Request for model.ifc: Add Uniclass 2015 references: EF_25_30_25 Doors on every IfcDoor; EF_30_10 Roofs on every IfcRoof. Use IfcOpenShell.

First a look at what the model holds.

```python
import ifcopenshell

model = ifcopenshell.open("model.ifc")
print(model.schema)
print("classifications:", [c.Name for c in model.by_type("IfcClassification")])
for ifc_class in ("IfcDoor", "IfcRoof", "IfcStair", "IfcWall", "IfcWindow"):
    print(ifc_class, len(model.by_type(ifc_class)))
```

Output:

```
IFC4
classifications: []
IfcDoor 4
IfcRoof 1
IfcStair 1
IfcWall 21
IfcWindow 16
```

```python
import ifcopenshell
import ifcopenshell.api.classification

model = ifcopenshell.open("model.ifc")

system = ifcopenshell.api.classification.add_classification(model, classification="Uniclass 2015")

codes = {
    "IfcDoor": ("EF_25_30_25", "Doors"),
    "IfcRoof": ("EF_30_10", "Roofs"),
}
for ifc_class, (code, name) in codes.items():
    products = model.by_type(ifc_class)
    ifcopenshell.api.classification.add_reference(
        model, products=products, classification=system, identification=code, name=name
    )
    print(code, len(products))

model.write("model_rev.ifc")
```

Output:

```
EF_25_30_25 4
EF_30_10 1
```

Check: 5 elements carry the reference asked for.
